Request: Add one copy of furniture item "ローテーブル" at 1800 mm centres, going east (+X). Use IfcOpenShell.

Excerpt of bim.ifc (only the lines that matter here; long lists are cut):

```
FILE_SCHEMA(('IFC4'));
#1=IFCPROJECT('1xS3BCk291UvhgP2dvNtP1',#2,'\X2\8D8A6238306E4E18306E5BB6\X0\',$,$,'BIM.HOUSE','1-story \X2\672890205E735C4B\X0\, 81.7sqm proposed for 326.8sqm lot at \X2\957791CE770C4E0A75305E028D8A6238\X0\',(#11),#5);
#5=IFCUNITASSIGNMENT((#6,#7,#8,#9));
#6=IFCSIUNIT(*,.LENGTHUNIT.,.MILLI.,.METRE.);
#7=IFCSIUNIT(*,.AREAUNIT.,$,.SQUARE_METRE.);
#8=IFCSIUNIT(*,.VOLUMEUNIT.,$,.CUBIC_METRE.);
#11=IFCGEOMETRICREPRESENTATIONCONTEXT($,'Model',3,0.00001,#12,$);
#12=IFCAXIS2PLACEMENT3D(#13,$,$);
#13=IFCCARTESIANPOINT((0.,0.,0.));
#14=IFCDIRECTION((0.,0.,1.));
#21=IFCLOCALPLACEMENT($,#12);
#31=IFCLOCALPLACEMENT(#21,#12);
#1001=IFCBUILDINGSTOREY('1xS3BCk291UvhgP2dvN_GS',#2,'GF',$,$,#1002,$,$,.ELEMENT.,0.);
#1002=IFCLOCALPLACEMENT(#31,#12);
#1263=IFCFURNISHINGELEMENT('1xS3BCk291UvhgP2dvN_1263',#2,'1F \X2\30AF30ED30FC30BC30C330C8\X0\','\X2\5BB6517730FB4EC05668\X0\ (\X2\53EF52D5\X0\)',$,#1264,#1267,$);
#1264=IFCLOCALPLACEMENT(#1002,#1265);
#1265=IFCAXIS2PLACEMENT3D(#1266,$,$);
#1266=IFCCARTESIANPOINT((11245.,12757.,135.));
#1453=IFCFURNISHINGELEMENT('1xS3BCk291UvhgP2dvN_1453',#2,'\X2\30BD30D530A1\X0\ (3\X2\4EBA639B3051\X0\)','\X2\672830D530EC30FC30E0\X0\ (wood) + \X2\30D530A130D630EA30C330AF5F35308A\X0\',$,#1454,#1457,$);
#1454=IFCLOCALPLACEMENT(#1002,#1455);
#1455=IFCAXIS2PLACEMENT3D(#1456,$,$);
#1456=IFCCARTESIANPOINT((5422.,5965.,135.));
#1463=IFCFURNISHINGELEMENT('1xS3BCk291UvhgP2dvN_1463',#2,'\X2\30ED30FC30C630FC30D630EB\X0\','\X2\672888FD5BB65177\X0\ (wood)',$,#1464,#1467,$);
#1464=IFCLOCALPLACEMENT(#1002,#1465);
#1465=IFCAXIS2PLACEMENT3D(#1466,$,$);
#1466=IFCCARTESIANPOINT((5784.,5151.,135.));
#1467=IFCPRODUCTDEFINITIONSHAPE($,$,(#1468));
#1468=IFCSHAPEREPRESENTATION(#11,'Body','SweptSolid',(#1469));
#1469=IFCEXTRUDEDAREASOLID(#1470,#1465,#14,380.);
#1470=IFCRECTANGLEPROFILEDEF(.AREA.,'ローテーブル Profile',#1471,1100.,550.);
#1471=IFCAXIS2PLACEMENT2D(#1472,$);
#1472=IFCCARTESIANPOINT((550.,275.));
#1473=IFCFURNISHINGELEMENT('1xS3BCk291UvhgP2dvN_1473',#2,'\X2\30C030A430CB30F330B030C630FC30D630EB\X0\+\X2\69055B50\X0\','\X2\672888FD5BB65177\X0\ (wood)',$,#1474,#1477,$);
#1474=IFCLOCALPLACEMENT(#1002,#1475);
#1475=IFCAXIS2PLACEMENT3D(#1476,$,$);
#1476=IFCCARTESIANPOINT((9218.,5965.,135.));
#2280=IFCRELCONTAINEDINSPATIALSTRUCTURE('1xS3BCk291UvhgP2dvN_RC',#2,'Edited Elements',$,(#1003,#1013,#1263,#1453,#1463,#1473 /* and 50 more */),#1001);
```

```python
import numpy as np
import ifcopenshell
import ifcopenshell.api.geometry
import ifcopenshell.api.root
import ifcopenshell.util.element
import ifcopenshell.util.placement
import ifcopenshell.util.unit

model = ifcopenshell.open("bim.ifc")
unit_scale = ifcopenshell.util.unit.calculate_unit_scale(model)


def reuse_history(source, copy):
    """copy_class also copies each property set's owner history, people and application; keep the originals."""
    for rel in copy.IsDefinedBy:
        if rel.is_a("IfcRelDefinesByProperties") and (history := rel.RelatingPropertyDefinition.OwnerHistory):
            rel.RelatingPropertyDefinition.OwnerHistory = source.OwnerHistory
            ifcopenshell.util.element.remove_deep2(model, history)


source = model.by_id(1463)
base = ifcopenshell.util.placement.get_local_placement(source.ObjectPlacement)
step = np.array([1.0, 0.0, 0.0]) * 1.8 / unit_scale

for i in range(1, 2):
    copy = ifcopenshell.api.root.copy_class(model, product=source)
    copy.Representation = ifcopenshell.util.element.copy_deep(
        model, source.Representation, exclude=["IfcGeometricRepresentationContext", "IfcRepresentationMap"]
    )
    reuse_history(source, copy)
    matrix = base.copy()
    matrix[:3, 3] += i * step
    print("added at", matrix[:3, 3].round(3) + 0.0)
    ifcopenshell.api.geometry.edit_object_placement(model, product=copy, matrix=matrix, is_si=False)

model.write("bim_v2.ifc")
```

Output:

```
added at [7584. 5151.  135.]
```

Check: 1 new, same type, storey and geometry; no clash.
